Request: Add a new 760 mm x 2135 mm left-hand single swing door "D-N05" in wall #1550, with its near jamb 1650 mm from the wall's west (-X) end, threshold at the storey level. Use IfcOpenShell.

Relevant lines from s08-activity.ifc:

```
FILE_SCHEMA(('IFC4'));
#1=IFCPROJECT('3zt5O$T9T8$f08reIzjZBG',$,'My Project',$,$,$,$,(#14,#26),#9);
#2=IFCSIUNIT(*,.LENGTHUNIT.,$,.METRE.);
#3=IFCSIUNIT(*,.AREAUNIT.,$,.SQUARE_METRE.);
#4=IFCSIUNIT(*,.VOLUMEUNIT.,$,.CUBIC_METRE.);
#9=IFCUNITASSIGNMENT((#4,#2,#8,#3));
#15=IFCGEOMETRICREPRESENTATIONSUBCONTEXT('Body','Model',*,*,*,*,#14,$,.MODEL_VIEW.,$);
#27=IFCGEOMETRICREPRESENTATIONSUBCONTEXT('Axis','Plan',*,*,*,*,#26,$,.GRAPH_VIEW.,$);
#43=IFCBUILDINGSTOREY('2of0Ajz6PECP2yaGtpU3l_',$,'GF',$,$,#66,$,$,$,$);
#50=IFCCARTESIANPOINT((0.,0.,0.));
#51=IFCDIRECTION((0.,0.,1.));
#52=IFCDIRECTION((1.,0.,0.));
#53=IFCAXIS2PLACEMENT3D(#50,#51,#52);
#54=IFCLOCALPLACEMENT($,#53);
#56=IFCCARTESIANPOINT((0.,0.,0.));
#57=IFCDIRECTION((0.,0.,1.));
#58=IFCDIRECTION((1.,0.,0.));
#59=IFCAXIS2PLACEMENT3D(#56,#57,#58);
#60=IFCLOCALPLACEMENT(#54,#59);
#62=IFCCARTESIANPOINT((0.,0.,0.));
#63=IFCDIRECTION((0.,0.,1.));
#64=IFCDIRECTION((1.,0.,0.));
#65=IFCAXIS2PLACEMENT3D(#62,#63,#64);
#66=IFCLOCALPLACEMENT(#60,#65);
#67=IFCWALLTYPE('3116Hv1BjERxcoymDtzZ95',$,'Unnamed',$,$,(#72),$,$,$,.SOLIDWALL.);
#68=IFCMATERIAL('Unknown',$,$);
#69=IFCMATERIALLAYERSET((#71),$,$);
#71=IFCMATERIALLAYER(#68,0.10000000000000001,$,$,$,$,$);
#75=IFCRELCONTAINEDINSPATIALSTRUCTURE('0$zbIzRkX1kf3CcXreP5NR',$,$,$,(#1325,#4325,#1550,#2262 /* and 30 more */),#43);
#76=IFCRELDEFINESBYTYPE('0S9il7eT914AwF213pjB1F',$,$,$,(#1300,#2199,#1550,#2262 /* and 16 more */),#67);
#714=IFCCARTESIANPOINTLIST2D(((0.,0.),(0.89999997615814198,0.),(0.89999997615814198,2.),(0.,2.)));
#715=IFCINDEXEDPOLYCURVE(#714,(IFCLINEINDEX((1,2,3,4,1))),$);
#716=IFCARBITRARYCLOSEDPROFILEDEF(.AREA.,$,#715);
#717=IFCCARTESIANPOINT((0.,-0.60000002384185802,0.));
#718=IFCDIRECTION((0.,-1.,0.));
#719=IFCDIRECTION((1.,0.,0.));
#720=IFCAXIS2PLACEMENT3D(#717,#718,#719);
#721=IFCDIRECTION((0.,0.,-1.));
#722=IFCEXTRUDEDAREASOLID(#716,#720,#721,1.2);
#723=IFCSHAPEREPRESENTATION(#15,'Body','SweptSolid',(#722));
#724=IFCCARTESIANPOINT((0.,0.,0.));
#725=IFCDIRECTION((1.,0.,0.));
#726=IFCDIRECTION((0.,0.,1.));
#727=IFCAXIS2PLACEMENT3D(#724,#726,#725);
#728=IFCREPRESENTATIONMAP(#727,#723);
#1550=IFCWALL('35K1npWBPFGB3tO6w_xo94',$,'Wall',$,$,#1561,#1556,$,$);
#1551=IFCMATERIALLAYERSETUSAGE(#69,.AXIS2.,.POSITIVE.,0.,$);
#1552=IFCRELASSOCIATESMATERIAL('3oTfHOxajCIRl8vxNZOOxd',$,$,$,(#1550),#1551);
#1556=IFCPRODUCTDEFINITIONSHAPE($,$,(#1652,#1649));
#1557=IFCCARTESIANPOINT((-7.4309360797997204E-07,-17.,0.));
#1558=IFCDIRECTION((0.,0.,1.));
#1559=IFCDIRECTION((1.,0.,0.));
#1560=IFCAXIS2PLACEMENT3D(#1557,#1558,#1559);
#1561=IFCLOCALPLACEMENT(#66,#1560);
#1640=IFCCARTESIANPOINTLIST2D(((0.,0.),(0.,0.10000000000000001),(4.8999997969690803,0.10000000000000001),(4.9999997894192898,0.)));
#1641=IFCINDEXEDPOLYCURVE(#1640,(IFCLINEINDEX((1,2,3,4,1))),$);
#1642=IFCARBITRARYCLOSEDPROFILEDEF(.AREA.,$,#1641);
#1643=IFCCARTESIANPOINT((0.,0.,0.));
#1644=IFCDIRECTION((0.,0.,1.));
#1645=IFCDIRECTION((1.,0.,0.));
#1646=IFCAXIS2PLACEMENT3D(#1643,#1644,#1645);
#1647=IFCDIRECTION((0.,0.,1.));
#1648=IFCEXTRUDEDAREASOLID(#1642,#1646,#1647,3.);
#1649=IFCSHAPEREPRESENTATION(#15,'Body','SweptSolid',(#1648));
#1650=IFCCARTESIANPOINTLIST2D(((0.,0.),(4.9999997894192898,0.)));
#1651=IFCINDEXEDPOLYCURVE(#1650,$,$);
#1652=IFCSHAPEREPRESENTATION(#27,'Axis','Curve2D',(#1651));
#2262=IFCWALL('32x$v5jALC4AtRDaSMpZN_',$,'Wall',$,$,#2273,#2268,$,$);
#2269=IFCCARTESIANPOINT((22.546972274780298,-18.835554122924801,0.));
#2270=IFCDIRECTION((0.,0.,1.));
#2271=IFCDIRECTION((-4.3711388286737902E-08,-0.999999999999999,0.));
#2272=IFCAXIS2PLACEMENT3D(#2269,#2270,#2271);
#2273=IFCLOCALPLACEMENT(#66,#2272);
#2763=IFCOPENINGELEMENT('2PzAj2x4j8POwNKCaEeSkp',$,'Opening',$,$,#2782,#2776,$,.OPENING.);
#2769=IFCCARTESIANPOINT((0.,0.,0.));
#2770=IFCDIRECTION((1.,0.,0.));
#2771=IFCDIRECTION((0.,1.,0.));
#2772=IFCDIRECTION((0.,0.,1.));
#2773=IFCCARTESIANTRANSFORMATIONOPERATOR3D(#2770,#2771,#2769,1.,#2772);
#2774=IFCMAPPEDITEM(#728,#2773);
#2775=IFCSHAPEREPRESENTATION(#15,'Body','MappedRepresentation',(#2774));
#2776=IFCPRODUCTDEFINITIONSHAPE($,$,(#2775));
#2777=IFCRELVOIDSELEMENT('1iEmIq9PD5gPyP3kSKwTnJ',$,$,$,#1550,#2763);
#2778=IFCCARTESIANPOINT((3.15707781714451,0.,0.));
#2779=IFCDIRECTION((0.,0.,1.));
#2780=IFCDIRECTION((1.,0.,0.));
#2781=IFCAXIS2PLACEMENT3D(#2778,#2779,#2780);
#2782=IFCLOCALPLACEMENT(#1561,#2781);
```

```python
import numpy as np
import ifcopenshell
import ifcopenshell.api.feature
import ifcopenshell.api.geometry
import ifcopenshell.api.root
import ifcopenshell.api.spatial
import ifcopenshell.geom
import ifcopenshell.util.element
import ifcopenshell.util.placement
import ifcopenshell.util.representation
import ifcopenshell.util.shape
import ifcopenshell.util.unit

model = ifcopenshell.open("s08-activity.ifc")
unit_scale = ifcopenshell.util.unit.calculate_unit_scale(model)
settings = ifcopenshell.geom.settings()


def volume(element):
    """Net volume in cubic metres, openings subtracted."""
    shape = ifcopenshell.geom.create_shape(settings, element)
    return ifcopenshell.util.shape.get_volume(shape.geometry)


wall = model.by_id(1550)
storey = ifcopenshell.util.element.get_container(wall, ifc_class="IfcBuildingStorey")
context = ifcopenshell.util.representation.get_context(model, "Model", "Body", "MODEL_VIEW")
before = volume(wall)

width, height, from_end, sill = 0.76, 2.135, 1.65, 0.0  # metres

# The wall runs along its own X axis, and the end named is its -X end.
wall_shape = ifcopenshell.geom.create_shape(settings, wall)
x, y, z = ifcopenshell.util.shape.get_vertices(wall_shape.geometry).T
start = x.min() + from_end
face, thickness = float(y.min()), float(y.max() - y.min())
wall_matrix = ifcopenshell.util.placement.get_local_placement(wall.ObjectPlacement)
level = ifcopenshell.util.placement.get_local_placement(storey.ObjectPlacement)[2, 3]


def in_wall(x, y):
    """Placement at x, y metres in the wall's axes, at sill height."""
    matrix = wall_matrix.copy()
    matrix[:, 3] = wall_matrix @ np.array([x / unit_scale, y / unit_scale, 0.0, 1.0])
    matrix[2, 3] = level + sill / unit_scale
    return matrix


# Opening: a box that overshoots both wall faces by 50 mm.
opening = ifcopenshell.api.root.create_entity(model, ifc_class="IfcOpeningElement", predefined_type="OPENING")
box = ifcopenshell.api.geometry.add_wall_representation(
    model, context=context, length=width, height=height, thickness=thickness + 0.1
)
ifcopenshell.api.geometry.assign_representation(model, product=opening, representation=box)
ifcopenshell.api.geometry.edit_object_placement(model, product=opening, matrix=in_wall(start, face - 0.05), is_si=False)
ifcopenshell.api.feature.add_feature(model, feature=opening, element=wall)

door = ifcopenshell.api.root.create_entity(model, ifc_class="IfcDoor", name="D-N05", predefined_type="DOOR")
door.OverallWidth, door.OverallHeight = width / unit_scale, height / unit_scale
door.OperationType = "SINGLE_SWING_LEFT"
body = ifcopenshell.api.geometry.add_door_representation(
    model,
    context=context,
    overall_width=door.OverallWidth,
    overall_height=door.OverallHeight,
    operation_type="SINGLE_SWING_LEFT",
    lining_properties={"LiningDepth": thickness / unit_scale, "ThresholdDepth": thickness / unit_scale},
)
ifcopenshell.api.geometry.assign_representation(model, product=door, representation=body)
ifcopenshell.api.spatial.assign_container(model, products=[door], relating_structure=storey)
ifcopenshell.api.feature.add_filling(model, opening=opening, element=door)

# The lining spans the wall, so the door starts at the wall face.
ifcopenshell.api.geometry.edit_object_placement(model, product=door, matrix=in_wall(start, face), is_si=False)

after = volume(wall)

print(f"wall volume {before:.3f} -> {after:.3f} m3")

model.write("s08-activity_edited.ifc")
```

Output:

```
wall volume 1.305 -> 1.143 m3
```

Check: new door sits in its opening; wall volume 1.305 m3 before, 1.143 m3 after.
